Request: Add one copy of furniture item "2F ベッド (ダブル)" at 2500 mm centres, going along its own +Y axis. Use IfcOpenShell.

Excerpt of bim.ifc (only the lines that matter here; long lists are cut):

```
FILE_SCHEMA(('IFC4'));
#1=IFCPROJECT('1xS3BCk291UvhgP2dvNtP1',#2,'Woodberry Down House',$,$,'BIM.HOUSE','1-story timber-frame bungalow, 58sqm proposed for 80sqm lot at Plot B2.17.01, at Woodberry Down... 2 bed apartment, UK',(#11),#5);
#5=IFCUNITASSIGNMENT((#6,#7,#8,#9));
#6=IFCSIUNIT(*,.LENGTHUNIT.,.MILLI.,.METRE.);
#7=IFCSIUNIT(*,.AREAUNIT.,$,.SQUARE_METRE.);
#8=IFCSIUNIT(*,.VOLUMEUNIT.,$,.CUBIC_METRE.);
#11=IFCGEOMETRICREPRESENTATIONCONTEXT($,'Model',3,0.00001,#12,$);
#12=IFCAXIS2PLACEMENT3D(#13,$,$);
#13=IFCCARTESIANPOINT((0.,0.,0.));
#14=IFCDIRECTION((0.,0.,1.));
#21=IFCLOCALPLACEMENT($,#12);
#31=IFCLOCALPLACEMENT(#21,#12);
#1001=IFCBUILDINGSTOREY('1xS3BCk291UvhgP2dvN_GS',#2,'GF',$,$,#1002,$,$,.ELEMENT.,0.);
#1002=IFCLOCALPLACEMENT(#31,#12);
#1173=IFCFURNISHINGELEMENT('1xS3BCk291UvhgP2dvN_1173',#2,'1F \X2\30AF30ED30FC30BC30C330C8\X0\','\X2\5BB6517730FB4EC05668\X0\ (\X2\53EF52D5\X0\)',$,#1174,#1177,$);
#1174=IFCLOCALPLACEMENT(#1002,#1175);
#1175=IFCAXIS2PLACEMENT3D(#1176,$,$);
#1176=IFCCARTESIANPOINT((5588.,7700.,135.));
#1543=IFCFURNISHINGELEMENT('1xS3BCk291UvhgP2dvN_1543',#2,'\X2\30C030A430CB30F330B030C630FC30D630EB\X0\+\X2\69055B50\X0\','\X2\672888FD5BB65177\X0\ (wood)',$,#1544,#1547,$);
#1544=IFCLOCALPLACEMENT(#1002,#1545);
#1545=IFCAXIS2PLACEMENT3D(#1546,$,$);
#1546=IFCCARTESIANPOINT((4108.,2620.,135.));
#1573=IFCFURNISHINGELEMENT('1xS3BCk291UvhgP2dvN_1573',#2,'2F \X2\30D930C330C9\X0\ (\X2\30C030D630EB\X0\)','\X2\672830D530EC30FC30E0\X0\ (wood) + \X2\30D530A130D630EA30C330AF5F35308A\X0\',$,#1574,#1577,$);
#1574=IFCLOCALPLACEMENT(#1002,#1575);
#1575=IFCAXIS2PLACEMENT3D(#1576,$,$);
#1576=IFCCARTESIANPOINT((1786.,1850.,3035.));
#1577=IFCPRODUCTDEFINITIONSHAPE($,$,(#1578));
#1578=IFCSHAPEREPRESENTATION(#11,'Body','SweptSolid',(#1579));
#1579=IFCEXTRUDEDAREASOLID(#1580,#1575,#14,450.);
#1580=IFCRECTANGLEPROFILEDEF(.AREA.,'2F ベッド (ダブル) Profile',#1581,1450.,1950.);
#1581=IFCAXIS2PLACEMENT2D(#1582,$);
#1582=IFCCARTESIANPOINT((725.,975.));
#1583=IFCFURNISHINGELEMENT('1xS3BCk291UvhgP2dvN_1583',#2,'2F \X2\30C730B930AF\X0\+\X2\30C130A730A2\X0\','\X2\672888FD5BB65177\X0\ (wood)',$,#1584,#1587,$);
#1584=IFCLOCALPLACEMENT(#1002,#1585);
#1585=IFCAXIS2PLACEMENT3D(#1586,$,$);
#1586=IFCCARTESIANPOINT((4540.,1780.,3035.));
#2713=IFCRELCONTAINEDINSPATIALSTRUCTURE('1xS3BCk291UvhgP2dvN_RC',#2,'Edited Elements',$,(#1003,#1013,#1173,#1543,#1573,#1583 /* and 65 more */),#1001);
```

```python
import ifcopenshell
import ifcopenshell.api.geometry
import ifcopenshell.api.root
import ifcopenshell.util.element
import ifcopenshell.util.placement
import ifcopenshell.util.unit

model = ifcopenshell.open("bim.ifc")
unit_scale = ifcopenshell.util.unit.calculate_unit_scale(model)


def reuse_history(source, copy):
    """copy_class also copies each property set's owner history, people and application; keep the originals."""
    for rel in copy.IsDefinedBy:
        if rel.is_a("IfcRelDefinesByProperties") and (history := rel.RelatingPropertyDefinition.OwnerHistory):
            rel.RelatingPropertyDefinition.OwnerHistory = source.OwnerHistory
            ifcopenshell.util.element.remove_deep2(model, history)


source = model.by_guid("1xS3BCk291UvhgP2dvN_1573")
base = ifcopenshell.util.placement.get_local_placement(source.ObjectPlacement)
step = base[:3, 1] * 2.5 / unit_scale

for i in range(1, 2):
    copy = ifcopenshell.api.root.copy_class(model, product=source)
    copy.Representation = ifcopenshell.util.element.copy_deep(
        model, source.Representation, exclude=["IfcGeometricRepresentationContext", "IfcRepresentationMap"]
    )
    reuse_history(source, copy)
    matrix = base.copy()
    matrix[:3, 3] += i * step
    print("added at", matrix[:3, 3].round(3) + 0.0)
    ifcopenshell.api.geometry.edit_object_placement(model, product=copy, matrix=matrix, is_si=False)

model.write("bim-out.ifc")
```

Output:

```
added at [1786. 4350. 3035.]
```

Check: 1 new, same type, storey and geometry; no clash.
